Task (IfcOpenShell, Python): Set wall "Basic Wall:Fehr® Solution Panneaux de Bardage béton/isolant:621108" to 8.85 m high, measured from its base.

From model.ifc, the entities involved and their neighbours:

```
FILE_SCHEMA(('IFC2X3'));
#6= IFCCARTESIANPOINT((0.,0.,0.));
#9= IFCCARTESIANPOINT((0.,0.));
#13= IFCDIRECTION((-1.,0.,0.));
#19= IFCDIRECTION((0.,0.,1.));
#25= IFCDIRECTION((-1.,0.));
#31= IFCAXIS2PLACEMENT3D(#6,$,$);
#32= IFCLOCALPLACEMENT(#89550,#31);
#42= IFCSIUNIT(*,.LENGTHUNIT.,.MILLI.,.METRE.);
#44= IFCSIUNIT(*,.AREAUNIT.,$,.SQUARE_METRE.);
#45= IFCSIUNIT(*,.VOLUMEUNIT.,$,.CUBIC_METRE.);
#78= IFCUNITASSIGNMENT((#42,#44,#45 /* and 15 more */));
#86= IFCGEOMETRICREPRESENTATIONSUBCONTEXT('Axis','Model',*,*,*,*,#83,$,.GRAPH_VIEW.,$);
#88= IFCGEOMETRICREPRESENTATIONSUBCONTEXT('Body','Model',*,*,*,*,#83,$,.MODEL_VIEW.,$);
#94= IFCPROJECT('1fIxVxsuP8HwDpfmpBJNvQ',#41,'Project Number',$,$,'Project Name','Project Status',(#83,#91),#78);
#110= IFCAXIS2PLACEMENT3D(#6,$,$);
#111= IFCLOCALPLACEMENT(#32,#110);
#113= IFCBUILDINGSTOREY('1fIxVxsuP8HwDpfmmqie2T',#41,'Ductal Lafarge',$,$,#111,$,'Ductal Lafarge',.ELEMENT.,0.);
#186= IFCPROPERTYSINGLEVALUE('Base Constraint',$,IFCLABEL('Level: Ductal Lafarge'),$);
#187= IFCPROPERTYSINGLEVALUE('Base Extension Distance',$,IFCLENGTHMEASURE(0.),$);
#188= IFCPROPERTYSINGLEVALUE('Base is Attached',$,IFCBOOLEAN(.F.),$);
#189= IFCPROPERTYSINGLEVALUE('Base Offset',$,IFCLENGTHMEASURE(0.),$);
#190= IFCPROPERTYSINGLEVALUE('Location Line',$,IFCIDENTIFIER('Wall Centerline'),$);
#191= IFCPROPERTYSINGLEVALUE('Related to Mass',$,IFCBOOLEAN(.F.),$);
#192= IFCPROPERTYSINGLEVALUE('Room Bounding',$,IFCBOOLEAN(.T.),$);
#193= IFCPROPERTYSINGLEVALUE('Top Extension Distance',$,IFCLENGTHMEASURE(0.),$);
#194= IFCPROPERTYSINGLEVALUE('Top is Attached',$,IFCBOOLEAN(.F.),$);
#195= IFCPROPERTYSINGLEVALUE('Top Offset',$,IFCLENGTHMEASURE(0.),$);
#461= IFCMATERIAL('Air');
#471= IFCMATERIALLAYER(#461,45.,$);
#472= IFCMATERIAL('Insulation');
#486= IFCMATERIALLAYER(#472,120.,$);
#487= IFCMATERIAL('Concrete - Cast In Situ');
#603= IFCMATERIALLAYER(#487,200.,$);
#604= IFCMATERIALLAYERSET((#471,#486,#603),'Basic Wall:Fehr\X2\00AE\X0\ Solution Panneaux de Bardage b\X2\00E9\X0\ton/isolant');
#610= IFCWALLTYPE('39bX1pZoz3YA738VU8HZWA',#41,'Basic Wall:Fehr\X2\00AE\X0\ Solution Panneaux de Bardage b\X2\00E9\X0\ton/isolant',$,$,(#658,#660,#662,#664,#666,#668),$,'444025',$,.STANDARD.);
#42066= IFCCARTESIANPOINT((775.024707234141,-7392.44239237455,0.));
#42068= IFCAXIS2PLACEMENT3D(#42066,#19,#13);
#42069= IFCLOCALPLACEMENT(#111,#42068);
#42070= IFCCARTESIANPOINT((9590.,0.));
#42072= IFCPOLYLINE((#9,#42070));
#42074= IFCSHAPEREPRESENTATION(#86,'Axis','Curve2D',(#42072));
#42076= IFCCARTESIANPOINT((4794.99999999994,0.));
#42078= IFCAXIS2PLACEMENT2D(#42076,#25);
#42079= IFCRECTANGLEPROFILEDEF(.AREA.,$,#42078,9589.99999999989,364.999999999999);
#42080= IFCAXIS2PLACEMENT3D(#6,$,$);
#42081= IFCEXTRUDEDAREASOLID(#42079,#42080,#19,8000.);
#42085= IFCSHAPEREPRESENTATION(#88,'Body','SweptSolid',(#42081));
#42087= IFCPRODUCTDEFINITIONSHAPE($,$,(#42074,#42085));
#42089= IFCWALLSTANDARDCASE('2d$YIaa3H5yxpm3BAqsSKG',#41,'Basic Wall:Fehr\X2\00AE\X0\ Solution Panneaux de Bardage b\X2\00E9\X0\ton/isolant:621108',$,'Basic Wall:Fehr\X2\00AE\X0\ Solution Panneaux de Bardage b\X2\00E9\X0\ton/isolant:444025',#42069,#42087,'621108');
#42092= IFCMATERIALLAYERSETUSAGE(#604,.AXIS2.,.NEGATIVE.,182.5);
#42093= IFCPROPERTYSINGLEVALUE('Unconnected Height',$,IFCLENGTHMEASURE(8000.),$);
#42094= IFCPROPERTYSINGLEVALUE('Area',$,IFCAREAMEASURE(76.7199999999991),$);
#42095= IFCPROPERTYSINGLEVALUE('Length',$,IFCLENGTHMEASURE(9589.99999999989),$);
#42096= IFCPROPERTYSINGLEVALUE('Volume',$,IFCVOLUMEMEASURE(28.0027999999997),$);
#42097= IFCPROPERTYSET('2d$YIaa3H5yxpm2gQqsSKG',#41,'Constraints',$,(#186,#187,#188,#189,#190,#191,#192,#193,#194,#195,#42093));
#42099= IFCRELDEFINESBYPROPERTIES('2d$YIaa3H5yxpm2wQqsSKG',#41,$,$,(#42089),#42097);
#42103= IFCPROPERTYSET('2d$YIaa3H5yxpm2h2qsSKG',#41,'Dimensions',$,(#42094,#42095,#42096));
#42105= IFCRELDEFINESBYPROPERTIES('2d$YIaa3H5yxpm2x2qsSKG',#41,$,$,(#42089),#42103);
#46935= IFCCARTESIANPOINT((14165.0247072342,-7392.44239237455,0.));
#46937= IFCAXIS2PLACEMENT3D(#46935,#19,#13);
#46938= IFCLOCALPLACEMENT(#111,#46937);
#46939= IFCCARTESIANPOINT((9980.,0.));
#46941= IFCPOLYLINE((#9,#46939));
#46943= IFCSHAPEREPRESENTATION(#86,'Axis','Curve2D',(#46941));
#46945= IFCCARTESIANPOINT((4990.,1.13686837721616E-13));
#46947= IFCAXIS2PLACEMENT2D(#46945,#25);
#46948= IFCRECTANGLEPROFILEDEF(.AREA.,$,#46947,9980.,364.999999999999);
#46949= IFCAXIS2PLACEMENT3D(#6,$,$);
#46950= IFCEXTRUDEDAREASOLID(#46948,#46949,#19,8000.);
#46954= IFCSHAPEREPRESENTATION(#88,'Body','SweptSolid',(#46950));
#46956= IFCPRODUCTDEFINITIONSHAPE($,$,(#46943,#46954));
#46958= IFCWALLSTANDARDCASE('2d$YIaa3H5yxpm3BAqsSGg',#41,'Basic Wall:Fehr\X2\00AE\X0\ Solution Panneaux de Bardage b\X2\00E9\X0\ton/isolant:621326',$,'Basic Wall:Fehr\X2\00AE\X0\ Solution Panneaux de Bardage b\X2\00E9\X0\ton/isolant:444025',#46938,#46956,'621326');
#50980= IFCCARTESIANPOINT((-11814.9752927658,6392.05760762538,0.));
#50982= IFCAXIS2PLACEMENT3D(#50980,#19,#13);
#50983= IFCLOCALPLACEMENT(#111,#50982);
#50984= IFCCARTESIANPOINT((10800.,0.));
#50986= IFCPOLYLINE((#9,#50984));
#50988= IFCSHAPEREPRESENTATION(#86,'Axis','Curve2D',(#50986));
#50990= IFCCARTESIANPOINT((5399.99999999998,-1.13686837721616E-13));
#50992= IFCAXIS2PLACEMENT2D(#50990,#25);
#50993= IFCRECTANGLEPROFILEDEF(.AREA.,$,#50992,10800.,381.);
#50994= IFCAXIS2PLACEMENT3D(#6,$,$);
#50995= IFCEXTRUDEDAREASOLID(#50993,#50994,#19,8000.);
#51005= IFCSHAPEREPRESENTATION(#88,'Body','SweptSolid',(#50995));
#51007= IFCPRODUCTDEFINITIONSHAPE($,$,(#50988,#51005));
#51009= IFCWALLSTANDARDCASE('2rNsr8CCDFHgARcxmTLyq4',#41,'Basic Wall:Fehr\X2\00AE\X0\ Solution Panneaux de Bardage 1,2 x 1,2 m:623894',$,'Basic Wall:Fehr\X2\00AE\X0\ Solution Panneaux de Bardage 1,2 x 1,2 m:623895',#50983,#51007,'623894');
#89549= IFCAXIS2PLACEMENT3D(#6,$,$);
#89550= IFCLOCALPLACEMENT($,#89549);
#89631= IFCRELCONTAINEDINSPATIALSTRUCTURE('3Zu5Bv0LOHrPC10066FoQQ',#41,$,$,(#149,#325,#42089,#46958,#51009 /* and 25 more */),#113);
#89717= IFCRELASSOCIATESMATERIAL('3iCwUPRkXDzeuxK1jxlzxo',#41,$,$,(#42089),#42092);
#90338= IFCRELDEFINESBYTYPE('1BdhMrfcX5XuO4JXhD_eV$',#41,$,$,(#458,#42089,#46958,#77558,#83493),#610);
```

```python
import ifcopenshell
import ifcopenshell.api.pset
import ifcopenshell.geom
import ifcopenshell.util.element
import ifcopenshell.util.representation
import ifcopenshell.util.shape
import ifcopenshell.util.unit

model = ifcopenshell.open("model.ifc")
area_scale = ifcopenshell.util.unit.calculate_unit_scale(model, "AREAUNIT")
volume_scale = ifcopenshell.util.unit.calculate_unit_scale(model, "VOLUMEUNIT")
settings = ifcopenshell.geom.settings()


def volume(element):
    """Net volume in cubic metres, openings subtracted."""
    shape = ifcopenshell.geom.create_shape(settings, element)
    return ifcopenshell.util.shape.get_volume(shape.geometry)


wall = model.by_guid("2d$YIaa3H5yxpm3BAqsSKG")
before = volume(wall)

body = ifcopenshell.util.representation.get_representation(wall, "Model", "Body")
solid = body.Items[0]
old_height = solid.Depth
solid.Depth = 8850.0
after = volume(wall)
thickness = 0.365  # wall thickness in metres

# Update the stored height, areas and volumes.
pset = model.by_id(ifcopenshell.util.element.get_pset(wall, "Constraints", should_inherit=False)["id"])
ifcopenshell.api.pset.edit_pset(model, pset=pset, properties={
    "Unconnected Height": model.create_entity("IfcLengthMeasure", solid.Depth),
})
pset = model.by_id(ifcopenshell.util.element.get_pset(wall, "Dimensions", should_inherit=False)["id"])
ifcopenshell.api.pset.edit_pset(model, pset=pset, properties={
    "Area": model.create_entity("IfcAreaMeasure", after / thickness / area_scale),
    "Volume": model.create_entity("IfcVolumeMeasure", after / volume_scale),
})

print(f"height {old_height:g} -> {solid.Depth:g}, volume {before:.3f} -> {after:.3f} m3")

model.write("model_updated.ifc")
```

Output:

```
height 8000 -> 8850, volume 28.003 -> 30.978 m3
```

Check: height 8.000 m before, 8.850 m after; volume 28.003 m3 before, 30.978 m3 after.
